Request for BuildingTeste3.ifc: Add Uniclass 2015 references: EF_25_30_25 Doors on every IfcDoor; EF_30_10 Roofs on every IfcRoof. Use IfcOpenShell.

First a look at what the model holds.

```python
import ifcopenshell

model = ifcopenshell.open("BuildingTeste3.ifc")
print(model.schema)
print("classifications:", [c.Name for c in model.by_type("IfcClassification")])
for ifc_class in ("IfcDoor", "IfcRoof", "IfcStair", "IfcWall", "IfcWindow"):
    print(ifc_class, len(model.by_type(ifc_class)))
```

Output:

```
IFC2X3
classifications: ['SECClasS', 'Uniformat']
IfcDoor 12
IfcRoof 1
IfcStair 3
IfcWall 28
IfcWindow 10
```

```python
import ifcopenshell
import ifcopenshell.api.classification

model = ifcopenshell.open("BuildingTeste3.ifc")

# IFC2X3 requires Source and Edition and has no link from the project to the system.
system = model.create_entity("IfcClassification", Source="NBS", Edition="2015", Name="Uniclass 2015")

codes = {
    "IfcDoor": ("EF_25_30_25", "Doors"),
    "IfcRoof": ("EF_30_10", "Roofs"),
}
for ifc_class, (code, name) in codes.items():
    products = model.by_type(ifc_class)
    ifcopenshell.api.classification.add_reference(
        model, products=products, classification=system, identification=code, name=name
    )
    print(code, len(products))

model.write("BuildingTeste3_edited.ifc")
```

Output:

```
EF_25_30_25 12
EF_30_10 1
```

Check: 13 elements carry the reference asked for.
